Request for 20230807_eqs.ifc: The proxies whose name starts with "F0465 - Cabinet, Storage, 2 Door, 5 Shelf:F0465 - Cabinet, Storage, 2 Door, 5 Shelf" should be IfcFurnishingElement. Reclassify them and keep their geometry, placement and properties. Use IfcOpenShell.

First a look at what the model holds.

```python
import re

import ifcopenshell

model = ifcopenshell.open("20230807_eqs.ifc")
print(model.schema)
seen = {}
for e in model.by_type("IfcBuildingElementProxy"):
    name = re.sub(r":\d+(:\d+)?$", "", e.Name or "")  # drop the element id that some exporters append
    seen[name] = seen.get(name, 0) + 1
for name, count in sorted(seen.items()):
    print(count, "x", name)
```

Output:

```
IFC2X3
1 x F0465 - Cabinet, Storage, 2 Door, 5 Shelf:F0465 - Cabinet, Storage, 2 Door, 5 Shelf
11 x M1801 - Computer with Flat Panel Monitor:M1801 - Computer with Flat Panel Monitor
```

```python
import ifcopenshell
import ifcopenshell.api.root

model = ifcopenshell.open("20230807_eqs.ifc")

proxies = [e.id() for e in model.by_type("IfcBuildingElementProxy") if (e.Name or "").startswith("F0465 - Cabinet, Storage, 2 Door, 5 Shelf:F0465 - Cabinet, Storage, 2 Door, 5 Shelf")]
for step_id in proxies:
    proxy = model.by_id(step_id)
    # Reclassifying a typed element also reclassifies its type and the type's other occurrences.
    if proxy.is_a("IfcBuildingElementProxy"):
        ifcopenshell.api.root.reassign_class(model, product=proxy, ifc_class="IfcFurnishingElement")

print(sum(model.by_id(i).is_a("IfcFurnishingElement") for i in proxies), "reclassified")

model.write("20230807_eqs_v2.ifc")
```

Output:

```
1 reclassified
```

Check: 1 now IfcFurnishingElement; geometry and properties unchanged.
